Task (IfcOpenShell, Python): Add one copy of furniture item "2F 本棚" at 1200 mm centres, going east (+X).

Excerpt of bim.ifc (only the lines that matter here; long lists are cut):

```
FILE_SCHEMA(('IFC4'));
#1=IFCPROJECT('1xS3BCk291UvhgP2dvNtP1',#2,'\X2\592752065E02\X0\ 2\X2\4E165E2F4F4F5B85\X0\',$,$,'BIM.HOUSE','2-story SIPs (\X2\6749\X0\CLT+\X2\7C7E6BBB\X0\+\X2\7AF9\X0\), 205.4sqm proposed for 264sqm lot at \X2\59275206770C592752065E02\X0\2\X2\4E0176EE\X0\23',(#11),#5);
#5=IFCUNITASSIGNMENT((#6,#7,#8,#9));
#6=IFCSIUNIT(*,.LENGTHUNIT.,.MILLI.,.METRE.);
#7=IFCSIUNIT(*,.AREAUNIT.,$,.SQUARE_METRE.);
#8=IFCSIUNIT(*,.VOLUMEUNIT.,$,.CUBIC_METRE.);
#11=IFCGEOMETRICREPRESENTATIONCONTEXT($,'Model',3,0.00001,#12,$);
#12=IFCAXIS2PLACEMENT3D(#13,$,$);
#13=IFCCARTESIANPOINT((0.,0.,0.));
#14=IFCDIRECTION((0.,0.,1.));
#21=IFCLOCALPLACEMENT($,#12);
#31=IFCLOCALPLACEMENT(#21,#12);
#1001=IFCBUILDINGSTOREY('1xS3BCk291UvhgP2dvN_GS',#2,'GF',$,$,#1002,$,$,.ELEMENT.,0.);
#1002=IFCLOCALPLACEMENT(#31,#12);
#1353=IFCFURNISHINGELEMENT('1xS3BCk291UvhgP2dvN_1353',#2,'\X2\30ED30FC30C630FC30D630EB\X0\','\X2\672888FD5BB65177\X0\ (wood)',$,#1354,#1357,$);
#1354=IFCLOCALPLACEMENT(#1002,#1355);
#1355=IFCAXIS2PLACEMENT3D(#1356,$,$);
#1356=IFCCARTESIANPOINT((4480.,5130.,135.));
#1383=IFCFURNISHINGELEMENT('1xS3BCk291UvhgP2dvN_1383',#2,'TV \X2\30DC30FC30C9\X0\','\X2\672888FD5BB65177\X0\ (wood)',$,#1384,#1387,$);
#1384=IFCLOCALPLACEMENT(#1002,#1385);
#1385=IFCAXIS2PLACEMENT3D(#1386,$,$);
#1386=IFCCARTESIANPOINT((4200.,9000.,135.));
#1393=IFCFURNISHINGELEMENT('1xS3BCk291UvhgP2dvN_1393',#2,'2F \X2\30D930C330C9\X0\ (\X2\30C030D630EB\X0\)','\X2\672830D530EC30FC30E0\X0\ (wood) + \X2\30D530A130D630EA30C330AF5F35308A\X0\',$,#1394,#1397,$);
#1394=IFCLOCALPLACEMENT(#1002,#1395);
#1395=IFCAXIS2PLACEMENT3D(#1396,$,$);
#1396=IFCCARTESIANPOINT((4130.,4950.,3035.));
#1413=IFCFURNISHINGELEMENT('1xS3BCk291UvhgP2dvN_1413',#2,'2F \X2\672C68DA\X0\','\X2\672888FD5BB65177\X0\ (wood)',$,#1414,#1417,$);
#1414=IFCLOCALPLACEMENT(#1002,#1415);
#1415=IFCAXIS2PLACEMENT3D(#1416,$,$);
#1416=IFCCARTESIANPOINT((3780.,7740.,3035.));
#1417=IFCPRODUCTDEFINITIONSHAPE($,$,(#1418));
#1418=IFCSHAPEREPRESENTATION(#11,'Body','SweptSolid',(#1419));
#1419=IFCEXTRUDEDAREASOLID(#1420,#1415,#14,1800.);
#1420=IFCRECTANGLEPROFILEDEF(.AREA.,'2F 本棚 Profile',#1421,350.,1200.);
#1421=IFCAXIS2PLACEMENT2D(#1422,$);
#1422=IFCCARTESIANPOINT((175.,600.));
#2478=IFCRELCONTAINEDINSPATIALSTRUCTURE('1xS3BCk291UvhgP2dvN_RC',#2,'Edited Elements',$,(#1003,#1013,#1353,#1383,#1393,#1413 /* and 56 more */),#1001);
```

```python
import numpy as np
import ifcopenshell
import ifcopenshell.api.geometry
import ifcopenshell.api.root
import ifcopenshell.util.element
import ifcopenshell.util.placement
import ifcopenshell.util.unit

model = ifcopenshell.open("bim.ifc")
unit_scale = ifcopenshell.util.unit.calculate_unit_scale(model)


def reuse_history(source, copy):
    """copy_class also copies each property set's owner history, people and application; keep the originals."""
    for rel in copy.IsDefinedBy:
        if rel.is_a("IfcRelDefinesByProperties") and (history := rel.RelatingPropertyDefinition.OwnerHistory):
            rel.RelatingPropertyDefinition.OwnerHistory = source.OwnerHistory
            ifcopenshell.util.element.remove_deep2(model, history)


source = model.by_guid("1xS3BCk291UvhgP2dvN_1413")
base = ifcopenshell.util.placement.get_local_placement(source.ObjectPlacement)
step = np.array([1.0, 0.0, 0.0]) * 1.2 / unit_scale

for i in range(1, 2):
    copy = ifcopenshell.api.root.copy_class(model, product=source)
    copy.Representation = ifcopenshell.util.element.copy_deep(
        model, source.Representation, exclude=["IfcGeometricRepresentationContext", "IfcRepresentationMap"]
    )
    reuse_history(source, copy)
    matrix = base.copy()
    matrix[:3, 3] += i * step
    print("added at", matrix[:3, 3].round(3) + 0.0)
    ifcopenshell.api.geometry.edit_object_placement(model, product=copy, matrix=matrix, is_si=False)

model.write("bim-out.ifc")
```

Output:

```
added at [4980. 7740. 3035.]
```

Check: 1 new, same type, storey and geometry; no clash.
